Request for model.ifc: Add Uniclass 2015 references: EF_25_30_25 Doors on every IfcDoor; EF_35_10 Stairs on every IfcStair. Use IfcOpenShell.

First a look at what the model holds.

```python
import ifcopenshell

model = ifcopenshell.open("model.ifc")
print(model.schema)
print("classifications:", [c.Name for c in model.by_type("IfcClassification")])
for ifc_class in ("IfcDoor", "IfcRoof", "IfcStair", "IfcWall", "IfcWindow"):
    print(ifc_class, len(model.by_type(ifc_class)))
```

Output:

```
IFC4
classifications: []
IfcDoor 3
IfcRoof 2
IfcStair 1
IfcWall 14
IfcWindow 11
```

```python
import ifcopenshell
import ifcopenshell.api.classification

model = ifcopenshell.open("model.ifc")

system = ifcopenshell.api.classification.add_classification(model, classification="Uniclass 2015")

codes = {
    "IfcDoor": ("EF_25_30_25", "Doors"),
    "IfcStair": ("EF_35_10", "Stairs"),
}
for ifc_class, (code, name) in codes.items():
    products = model.by_type(ifc_class)
    ifcopenshell.api.classification.add_reference(
        model, products=products, classification=system, identification=code, name=name
    )
    print(code, len(products))

model.write("model_rev.ifc")
```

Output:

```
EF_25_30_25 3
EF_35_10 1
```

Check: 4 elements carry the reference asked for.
